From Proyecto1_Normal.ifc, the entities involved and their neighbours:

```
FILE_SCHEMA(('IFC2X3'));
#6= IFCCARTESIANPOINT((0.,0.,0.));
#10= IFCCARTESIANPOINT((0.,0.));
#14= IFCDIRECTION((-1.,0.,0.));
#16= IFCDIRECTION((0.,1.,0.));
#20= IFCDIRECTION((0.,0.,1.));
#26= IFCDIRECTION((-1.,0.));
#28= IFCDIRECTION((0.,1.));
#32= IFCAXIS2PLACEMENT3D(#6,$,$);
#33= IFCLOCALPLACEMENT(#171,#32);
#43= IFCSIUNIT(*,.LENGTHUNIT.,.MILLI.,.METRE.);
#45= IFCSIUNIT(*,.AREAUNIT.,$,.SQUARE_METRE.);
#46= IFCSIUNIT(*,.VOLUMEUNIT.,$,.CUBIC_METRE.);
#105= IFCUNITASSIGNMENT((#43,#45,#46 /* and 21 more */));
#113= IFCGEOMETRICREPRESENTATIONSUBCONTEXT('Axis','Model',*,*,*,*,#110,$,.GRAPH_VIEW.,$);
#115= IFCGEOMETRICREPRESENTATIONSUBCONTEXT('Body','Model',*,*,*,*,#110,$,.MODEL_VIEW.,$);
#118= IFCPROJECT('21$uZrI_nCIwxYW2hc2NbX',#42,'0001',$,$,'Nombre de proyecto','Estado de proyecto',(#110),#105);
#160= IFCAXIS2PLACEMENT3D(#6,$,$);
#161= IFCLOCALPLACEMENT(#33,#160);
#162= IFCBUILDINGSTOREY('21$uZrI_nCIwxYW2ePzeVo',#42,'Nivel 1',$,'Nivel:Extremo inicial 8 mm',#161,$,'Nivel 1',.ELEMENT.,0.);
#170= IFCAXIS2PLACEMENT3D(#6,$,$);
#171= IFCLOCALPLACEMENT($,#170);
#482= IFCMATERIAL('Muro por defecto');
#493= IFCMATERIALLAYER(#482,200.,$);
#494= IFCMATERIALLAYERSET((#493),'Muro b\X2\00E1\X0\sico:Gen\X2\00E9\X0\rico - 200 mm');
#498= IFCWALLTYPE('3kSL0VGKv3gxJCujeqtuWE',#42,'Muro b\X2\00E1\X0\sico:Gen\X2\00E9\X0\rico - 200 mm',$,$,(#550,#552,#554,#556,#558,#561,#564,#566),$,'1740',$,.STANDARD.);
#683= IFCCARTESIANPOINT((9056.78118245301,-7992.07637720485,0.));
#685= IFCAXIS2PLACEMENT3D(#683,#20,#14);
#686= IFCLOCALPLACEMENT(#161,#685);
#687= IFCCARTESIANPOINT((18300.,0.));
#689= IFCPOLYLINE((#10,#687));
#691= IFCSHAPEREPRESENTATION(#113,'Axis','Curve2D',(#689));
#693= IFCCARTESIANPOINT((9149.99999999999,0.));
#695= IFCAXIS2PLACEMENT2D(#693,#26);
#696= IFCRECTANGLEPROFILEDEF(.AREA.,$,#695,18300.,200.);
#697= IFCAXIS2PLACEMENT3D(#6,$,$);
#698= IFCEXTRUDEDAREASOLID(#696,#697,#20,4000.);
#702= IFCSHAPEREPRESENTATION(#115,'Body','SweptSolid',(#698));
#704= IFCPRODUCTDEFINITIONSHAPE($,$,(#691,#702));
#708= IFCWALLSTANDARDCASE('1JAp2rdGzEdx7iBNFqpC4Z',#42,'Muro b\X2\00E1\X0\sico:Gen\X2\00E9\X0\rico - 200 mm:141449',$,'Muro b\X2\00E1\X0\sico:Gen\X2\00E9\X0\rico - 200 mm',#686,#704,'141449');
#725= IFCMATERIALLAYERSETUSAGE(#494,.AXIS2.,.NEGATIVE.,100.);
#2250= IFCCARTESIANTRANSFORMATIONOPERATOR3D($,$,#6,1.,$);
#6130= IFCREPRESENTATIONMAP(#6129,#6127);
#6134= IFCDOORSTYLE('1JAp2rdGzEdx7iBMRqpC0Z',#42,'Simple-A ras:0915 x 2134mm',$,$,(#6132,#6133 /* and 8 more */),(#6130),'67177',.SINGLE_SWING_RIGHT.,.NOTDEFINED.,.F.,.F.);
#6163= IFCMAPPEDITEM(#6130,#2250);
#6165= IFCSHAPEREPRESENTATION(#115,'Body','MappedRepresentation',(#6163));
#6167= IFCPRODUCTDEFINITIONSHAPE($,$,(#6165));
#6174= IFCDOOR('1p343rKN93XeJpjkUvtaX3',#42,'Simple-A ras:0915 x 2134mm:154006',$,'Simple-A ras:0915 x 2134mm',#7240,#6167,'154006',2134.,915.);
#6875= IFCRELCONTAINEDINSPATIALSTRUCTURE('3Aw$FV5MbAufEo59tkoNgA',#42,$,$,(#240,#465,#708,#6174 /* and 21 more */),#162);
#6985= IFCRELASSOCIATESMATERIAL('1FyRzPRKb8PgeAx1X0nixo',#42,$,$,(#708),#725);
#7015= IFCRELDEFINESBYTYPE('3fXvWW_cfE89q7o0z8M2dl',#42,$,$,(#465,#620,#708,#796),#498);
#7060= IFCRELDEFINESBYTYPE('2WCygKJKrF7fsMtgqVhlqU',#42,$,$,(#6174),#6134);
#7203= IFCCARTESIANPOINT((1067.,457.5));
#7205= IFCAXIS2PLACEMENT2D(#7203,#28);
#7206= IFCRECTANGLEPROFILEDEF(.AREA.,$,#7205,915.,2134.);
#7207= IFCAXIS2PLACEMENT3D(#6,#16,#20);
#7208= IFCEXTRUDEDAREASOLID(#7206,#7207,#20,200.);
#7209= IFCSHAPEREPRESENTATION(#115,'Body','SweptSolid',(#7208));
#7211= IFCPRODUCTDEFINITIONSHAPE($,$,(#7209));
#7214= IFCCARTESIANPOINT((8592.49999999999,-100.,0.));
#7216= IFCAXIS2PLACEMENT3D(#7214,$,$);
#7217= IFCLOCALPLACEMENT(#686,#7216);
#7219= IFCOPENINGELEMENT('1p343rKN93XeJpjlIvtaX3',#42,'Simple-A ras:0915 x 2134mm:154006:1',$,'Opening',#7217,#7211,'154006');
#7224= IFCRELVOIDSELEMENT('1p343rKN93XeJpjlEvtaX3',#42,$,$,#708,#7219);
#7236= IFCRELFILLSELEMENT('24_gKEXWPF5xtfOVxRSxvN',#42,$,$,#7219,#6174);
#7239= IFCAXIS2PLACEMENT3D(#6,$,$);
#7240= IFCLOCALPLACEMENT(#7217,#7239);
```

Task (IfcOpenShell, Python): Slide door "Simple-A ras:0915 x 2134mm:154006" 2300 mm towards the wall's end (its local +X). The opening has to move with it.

```python
import ifcopenshell
import ifcopenshell.api.geometry
import ifcopenshell.util.placement
import ifcopenshell.util.unit

model = ifcopenshell.open("Proyecto1_Normal.ifc")
unit_scale = ifcopenshell.util.unit.calculate_unit_scale(model)

door = model.by_guid("1p343rKN93XeJpjkUvtaX3")
opening = door.FillsVoids[0].RelatingOpeningElement
wall = opening.VoidsElements[0].RelatingBuildingElement

wall_matrix = ifcopenshell.util.placement.get_local_placement(wall.ObjectPlacement)
shift = wall_matrix[:3, 0] * 2.3 / unit_scale
before = ifcopenshell.util.placement.get_local_placement(door.ObjectPlacement)[:3, 3].copy()

# The door is placed relative to its opening, so it follows when the opening moves.
matrix = ifcopenshell.util.placement.get_local_placement(opening.ObjectPlacement)
matrix[:3, 3] += shift
ifcopenshell.api.geometry.edit_object_placement(
    model, product=opening, matrix=matrix, is_si=False, should_transform_children=True
)

after = ifcopenshell.util.placement.get_local_placement(door.ObjectPlacement)[:3, 3]
print("door moved by", (after - before).round(3) + 0.0)

model.write("Proyecto1_Normal_edited.ifc")
```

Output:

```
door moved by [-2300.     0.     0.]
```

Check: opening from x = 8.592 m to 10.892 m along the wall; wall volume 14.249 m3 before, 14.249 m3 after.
